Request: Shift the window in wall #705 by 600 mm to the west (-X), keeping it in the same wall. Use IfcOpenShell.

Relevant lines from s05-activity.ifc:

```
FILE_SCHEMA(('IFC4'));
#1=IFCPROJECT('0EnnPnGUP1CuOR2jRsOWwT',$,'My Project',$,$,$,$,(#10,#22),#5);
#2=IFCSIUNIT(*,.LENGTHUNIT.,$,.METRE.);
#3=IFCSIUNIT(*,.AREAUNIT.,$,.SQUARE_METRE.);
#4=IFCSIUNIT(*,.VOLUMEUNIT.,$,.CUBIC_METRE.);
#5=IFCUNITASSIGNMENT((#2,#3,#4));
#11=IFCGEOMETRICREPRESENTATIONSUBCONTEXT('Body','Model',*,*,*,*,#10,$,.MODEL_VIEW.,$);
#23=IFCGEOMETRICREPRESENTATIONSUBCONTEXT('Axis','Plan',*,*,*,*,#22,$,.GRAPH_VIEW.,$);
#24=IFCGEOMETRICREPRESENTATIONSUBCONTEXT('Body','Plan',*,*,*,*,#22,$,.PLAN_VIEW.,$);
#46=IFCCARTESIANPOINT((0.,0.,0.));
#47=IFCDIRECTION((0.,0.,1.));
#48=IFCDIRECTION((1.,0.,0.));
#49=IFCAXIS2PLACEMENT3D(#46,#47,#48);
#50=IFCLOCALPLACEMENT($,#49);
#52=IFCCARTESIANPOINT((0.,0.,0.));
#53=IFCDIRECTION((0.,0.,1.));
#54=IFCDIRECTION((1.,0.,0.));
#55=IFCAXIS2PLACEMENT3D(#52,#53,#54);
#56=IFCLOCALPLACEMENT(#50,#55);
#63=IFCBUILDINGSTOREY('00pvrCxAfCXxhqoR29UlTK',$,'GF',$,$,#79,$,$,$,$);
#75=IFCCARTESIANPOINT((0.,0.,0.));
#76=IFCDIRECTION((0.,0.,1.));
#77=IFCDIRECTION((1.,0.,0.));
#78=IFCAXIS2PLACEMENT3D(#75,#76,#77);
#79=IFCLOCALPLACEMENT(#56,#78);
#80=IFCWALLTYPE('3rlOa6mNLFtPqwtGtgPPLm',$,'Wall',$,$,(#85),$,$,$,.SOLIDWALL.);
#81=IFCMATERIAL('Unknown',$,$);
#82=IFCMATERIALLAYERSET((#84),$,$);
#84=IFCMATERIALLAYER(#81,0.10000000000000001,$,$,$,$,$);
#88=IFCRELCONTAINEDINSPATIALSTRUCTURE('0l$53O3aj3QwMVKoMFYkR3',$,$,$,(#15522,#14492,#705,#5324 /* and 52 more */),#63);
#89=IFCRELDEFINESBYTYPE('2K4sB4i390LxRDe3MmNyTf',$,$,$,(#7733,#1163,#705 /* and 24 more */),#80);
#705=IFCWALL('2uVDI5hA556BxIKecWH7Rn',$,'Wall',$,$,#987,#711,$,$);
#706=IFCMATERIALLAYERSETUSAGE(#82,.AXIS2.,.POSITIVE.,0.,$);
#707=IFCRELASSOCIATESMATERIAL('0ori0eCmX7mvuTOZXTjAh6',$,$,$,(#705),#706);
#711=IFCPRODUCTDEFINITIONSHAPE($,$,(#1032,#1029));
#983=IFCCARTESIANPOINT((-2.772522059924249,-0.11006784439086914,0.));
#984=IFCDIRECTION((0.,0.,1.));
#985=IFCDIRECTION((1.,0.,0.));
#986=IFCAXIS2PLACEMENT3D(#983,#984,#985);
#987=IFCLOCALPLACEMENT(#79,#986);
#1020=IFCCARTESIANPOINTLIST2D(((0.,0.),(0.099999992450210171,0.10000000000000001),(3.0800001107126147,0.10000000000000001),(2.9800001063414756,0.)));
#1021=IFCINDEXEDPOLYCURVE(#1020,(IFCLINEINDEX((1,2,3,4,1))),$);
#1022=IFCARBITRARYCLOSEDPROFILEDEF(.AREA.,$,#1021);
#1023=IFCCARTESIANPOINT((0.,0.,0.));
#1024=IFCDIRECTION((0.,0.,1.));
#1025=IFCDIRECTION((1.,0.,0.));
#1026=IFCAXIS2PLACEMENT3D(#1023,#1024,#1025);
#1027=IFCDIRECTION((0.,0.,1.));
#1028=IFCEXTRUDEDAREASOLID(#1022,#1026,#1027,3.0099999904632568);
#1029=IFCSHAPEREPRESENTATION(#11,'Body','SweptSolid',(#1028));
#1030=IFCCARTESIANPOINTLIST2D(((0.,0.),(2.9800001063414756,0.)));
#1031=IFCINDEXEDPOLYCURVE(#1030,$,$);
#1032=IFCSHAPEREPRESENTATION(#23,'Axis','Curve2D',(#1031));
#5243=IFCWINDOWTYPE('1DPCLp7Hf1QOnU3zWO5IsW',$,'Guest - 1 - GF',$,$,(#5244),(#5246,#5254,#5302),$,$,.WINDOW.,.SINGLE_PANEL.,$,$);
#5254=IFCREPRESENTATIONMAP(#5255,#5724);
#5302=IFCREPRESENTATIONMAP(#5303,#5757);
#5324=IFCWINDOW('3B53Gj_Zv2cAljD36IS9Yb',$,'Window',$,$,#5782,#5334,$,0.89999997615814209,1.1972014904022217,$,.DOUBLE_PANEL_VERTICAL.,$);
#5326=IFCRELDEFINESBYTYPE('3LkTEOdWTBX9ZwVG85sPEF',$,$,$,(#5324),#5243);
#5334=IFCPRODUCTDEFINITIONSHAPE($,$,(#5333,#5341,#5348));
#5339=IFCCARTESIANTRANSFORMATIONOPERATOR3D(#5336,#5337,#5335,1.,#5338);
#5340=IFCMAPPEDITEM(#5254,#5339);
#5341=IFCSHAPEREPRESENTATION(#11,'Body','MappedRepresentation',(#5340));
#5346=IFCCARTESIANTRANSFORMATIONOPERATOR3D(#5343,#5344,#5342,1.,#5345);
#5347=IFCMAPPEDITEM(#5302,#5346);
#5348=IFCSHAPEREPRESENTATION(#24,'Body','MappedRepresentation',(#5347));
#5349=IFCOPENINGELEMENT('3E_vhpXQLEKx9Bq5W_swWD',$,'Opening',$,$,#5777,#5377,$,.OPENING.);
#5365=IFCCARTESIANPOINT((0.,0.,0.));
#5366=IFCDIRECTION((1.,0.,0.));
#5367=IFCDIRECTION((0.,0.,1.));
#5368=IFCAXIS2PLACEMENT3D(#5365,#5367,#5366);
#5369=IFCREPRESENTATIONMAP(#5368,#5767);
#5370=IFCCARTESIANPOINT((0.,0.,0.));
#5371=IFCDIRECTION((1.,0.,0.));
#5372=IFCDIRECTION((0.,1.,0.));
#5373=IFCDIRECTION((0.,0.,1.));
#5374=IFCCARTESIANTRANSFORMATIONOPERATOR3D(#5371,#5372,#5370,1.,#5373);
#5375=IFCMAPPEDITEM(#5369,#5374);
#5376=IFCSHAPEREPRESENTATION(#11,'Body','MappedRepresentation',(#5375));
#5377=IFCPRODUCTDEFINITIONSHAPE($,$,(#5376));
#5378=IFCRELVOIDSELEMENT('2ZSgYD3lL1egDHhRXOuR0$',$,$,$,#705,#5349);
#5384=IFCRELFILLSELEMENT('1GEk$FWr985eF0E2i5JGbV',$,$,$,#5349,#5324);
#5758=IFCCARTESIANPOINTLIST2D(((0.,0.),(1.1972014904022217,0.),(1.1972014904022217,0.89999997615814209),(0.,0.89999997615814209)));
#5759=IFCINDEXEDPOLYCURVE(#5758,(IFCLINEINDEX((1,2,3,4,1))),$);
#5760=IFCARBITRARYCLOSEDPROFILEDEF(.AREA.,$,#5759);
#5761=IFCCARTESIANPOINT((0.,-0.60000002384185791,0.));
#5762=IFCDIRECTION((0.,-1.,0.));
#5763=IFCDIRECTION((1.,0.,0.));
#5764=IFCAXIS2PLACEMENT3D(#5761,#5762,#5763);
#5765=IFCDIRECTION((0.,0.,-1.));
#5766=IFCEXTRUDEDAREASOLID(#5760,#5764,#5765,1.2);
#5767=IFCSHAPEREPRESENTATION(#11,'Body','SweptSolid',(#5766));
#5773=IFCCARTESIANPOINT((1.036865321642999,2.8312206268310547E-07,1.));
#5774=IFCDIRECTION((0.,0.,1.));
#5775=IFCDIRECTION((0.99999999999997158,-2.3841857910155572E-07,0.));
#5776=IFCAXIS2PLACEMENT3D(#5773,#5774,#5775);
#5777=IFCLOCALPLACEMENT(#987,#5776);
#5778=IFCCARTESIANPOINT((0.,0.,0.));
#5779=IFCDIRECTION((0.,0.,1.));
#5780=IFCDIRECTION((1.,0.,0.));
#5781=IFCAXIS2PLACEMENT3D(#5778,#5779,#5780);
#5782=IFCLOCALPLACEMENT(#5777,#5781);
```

```python
import ifcopenshell
import ifcopenshell.api.geometry
import ifcopenshell.util.placement
import ifcopenshell.util.unit

model = ifcopenshell.open("s05-activity.ifc")
unit_scale = ifcopenshell.util.unit.calculate_unit_scale(model)

window = model.by_guid("3B53Gj_Zv2cAljD36IS9Yb")
opening = window.FillsVoids[0].RelatingOpeningElement
wall = opening.VoidsElements[0].RelatingBuildingElement

wall_matrix = ifcopenshell.util.placement.get_local_placement(wall.ObjectPlacement)
shift = wall_matrix[:3, 0] * -0.6 / unit_scale
before = ifcopenshell.util.placement.get_local_placement(window.ObjectPlacement)[:3, 3].copy()

# The window is placed relative to its opening, so it follows when the opening moves.
matrix = ifcopenshell.util.placement.get_local_placement(opening.ObjectPlacement)
matrix[:3, 3] += shift
ifcopenshell.api.geometry.edit_object_placement(
    model, product=opening, matrix=matrix, is_si=False, should_transform_children=True
)

after = ifcopenshell.util.placement.get_local_placement(window.ObjectPlacement)[:3, 3]
print("window moved by", (after - before).round(3) + 0.0)

model.write("s05-activity_edited.ifc")
```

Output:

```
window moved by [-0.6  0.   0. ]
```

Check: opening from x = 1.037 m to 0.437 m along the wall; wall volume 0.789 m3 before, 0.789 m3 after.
